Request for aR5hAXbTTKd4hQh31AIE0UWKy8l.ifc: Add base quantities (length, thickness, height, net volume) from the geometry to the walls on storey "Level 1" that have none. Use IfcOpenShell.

First a look at what the model holds.

```python
import ifcopenshell
import ifcopenshell.util.element
import ifcopenshell.util.unit

model = ifcopenshell.open("aR5hAXbTTKd4hQh31AIE0UWKy8l.ifc")
print(model.schema)
for unit_type in ("LENGTHUNIT", "AREAUNIT", "VOLUMEUNIT"):
    print(unit_type, ifcopenshell.util.unit.calculate_unit_scale(model, unit_type))
storey = next(s for s in model.by_type("IfcBuildingStorey") if s.Name == "Level 1")
walls = [e for e in ifcopenshell.util.element.get_decomposition(storey) if e.is_a("IfcWall")]
for e in sorted(walls, key=lambda e: e.id()):
    print(e.id(), e.is_a(), e.Name, list(ifcopenshell.util.element.get_psets(e, qtos_only=True)), sep=" | ")
```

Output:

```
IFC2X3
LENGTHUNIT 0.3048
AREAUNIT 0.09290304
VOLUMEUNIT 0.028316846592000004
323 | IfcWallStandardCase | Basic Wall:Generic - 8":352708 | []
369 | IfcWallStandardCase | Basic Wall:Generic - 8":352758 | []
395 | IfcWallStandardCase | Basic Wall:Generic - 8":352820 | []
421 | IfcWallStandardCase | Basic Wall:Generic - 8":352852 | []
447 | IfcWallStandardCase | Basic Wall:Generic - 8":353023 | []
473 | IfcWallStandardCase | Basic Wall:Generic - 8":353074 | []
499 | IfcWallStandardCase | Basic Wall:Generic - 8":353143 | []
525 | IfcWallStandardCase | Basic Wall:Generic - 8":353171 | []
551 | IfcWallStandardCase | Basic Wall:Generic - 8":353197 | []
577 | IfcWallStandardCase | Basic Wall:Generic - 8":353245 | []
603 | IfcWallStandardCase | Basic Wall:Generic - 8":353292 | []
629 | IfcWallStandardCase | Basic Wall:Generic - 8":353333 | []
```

```python
import ifcopenshell
import ifcopenshell.api.pset
import ifcopenshell.geom
import ifcopenshell.util.element
import ifcopenshell.util.shape
import ifcopenshell.util.unit

model = ifcopenshell.open("aR5hAXbTTKd4hQh31AIE0UWKy8l.ifc")
unit_scale = ifcopenshell.util.unit.calculate_unit_scale(model)
volume_scale = ifcopenshell.util.unit.calculate_unit_scale(model, "VOLUMEUNIT")
settings = ifcopenshell.geom.settings()

storey = next(s for s in model.by_type("IfcBuildingStorey") if s.Name == "Level 1")
walls = [e for e in ifcopenshell.util.element.get_decomposition(storey) if e.is_a("IfcWall")]

for e in sorted(walls, key=lambda e: e.id()):
    if ifcopenshell.util.element.get_psets(e, qtos_only=True, should_inherit=False):
        continue
    # Geometry comes back in metres, in the element's own axes.
    shape = ifcopenshell.geom.create_shape(settings, e)
    values = {
        "Length": ifcopenshell.util.shape.get_x(shape.geometry) / unit_scale,
        "Width": ifcopenshell.util.shape.get_y(shape.geometry) / unit_scale,
        "Height": ifcopenshell.util.shape.get_z(shape.geometry) / unit_scale,
        "NetVolume": ifcopenshell.util.shape.get_volume(shape.geometry) / volume_scale,
    }
    qto = ifcopenshell.api.pset.add_qto(model, product=e, name="BaseQuantities")
    ifcopenshell.api.pset.edit_qto(model, qto=qto, properties=values)
    print(e.id(), {k: round(v, 3) for k, v in values.items()})

model.write("aR5hAXbTTKd4hQh31AIE0UWKy8l_v2.ifc")
```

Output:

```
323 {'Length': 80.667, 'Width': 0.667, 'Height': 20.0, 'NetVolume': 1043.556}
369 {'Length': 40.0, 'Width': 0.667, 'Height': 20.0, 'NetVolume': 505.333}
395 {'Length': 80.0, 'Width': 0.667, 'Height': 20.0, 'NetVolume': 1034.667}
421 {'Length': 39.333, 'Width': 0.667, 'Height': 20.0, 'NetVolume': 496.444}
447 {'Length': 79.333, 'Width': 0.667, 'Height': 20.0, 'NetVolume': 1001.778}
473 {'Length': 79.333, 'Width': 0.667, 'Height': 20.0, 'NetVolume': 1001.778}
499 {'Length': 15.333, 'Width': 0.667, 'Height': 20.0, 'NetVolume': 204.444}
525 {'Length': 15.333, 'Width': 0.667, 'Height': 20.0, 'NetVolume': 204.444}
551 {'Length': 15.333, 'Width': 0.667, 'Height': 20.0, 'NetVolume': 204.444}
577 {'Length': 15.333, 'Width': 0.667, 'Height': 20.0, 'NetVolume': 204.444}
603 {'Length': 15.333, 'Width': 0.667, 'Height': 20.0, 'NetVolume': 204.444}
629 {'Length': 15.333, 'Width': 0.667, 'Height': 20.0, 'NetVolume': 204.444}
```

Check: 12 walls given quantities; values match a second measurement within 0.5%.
